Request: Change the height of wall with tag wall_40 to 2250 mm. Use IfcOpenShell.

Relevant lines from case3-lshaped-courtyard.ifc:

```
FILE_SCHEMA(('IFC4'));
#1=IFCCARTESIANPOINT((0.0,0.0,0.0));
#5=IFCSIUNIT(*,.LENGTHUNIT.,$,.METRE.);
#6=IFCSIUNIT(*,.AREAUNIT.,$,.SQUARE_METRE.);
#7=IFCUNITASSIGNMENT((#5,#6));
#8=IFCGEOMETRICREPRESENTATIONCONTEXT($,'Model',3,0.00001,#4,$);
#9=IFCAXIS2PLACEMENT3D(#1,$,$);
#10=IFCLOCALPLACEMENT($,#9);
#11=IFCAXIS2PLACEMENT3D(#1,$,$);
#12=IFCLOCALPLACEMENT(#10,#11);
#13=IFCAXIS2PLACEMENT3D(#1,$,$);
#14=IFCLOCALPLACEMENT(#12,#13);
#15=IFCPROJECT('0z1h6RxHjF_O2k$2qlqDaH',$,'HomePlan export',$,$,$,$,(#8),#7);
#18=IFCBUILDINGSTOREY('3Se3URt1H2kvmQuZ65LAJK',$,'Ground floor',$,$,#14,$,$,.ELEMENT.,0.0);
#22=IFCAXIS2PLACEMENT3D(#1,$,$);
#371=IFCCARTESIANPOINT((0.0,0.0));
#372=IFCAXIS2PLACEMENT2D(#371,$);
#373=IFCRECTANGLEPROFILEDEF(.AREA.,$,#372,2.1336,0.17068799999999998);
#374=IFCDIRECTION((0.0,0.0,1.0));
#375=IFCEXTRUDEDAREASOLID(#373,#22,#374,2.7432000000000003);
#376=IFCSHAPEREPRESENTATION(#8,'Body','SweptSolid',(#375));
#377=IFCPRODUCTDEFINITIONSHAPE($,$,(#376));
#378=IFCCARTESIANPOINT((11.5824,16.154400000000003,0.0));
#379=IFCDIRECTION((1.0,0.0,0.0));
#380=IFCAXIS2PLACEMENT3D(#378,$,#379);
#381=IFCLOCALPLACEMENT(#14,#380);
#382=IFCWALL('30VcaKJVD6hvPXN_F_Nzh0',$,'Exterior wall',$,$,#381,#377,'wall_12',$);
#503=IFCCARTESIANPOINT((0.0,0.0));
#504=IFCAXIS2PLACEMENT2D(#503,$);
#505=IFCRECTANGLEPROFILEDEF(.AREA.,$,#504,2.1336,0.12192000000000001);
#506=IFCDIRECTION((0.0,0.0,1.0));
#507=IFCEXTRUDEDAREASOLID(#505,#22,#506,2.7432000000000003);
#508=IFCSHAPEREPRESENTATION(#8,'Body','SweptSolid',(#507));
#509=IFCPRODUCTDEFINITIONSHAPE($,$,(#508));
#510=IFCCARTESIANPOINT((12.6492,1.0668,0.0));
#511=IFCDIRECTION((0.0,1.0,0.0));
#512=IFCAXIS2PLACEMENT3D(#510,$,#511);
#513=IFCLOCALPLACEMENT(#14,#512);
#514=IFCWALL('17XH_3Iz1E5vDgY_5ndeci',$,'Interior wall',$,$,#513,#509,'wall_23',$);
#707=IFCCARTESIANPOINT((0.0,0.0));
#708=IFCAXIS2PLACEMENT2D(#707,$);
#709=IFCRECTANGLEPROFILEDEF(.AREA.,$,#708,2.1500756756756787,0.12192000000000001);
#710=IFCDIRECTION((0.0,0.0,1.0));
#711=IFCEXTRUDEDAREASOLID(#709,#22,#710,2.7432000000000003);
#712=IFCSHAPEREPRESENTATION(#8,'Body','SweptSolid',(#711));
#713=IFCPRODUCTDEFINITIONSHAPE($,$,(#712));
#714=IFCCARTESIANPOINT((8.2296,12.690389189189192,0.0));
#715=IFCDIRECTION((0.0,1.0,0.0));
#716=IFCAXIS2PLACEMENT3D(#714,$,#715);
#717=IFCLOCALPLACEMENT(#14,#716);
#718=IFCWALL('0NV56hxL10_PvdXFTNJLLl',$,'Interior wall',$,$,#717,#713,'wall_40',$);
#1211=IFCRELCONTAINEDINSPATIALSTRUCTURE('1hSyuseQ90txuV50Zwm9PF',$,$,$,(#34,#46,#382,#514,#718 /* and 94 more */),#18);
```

```python
import ifcopenshell
import ifcopenshell.geom
import ifcopenshell.util.shape
import ifcopenshell.util.unit

model = ifcopenshell.open("case3-lshaped-courtyard.ifc")
unit_scale = ifcopenshell.util.unit.calculate_unit_scale(model)
settings = ifcopenshell.geom.settings()


def volume(element):
    """Net volume in cubic metres, openings subtracted."""
    shape = ifcopenshell.geom.create_shape(settings, element)
    return ifcopenshell.util.shape.get_volume(shape.geometry)


wall = model.by_id(718)
before = volume(wall)

body = next(r for r in wall.Representation.Representations if r.RepresentationIdentifier == "Body")
solid = body.Items[0]
old_height = solid.Depth
solid.Depth = 2.25 / unit_scale
after = volume(wall)

print(f"height {old_height:g} -> {solid.Depth:g}, volume {before:.3f} -> {after:.3f} m3")

model.write("case3-lshaped-courtyard_rev.ifc")
```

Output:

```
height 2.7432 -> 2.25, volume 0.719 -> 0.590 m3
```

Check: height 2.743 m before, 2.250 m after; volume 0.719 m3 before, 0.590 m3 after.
